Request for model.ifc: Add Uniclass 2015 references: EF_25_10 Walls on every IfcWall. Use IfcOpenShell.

First a look at what the model holds.

```python
import ifcopenshell

model = ifcopenshell.open("model.ifc")
print(model.schema)
print("classifications:", [c.Name for c in model.by_type("IfcClassification")])
for ifc_class in ("IfcDoor", "IfcRoof", "IfcStair", "IfcWall", "IfcWindow"):
    print(ifc_class, len(model.by_type(ifc_class)))
```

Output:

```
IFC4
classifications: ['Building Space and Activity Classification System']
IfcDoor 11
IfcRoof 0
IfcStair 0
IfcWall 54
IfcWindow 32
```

```python
import ifcopenshell
import ifcopenshell.api.classification

model = ifcopenshell.open("model.ifc")

system = ifcopenshell.api.classification.add_classification(model, classification="Uniclass 2015")

codes = {
    "IfcWall": ("EF_25_10", "Walls"),
}
for ifc_class, (code, name) in codes.items():
    products = model.by_type(ifc_class)
    ifcopenshell.api.classification.add_reference(
        model, products=products, classification=system, identification=code, name=name
    )
    print(code, len(products))

model.write("model-out.ifc")
```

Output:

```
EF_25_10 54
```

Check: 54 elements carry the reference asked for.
